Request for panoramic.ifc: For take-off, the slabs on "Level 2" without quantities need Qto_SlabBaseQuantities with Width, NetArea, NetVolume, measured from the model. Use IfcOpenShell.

First a look at what the model holds.

```python
import ifcopenshell
import ifcopenshell.util.element
import ifcopenshell.util.unit

model = ifcopenshell.open("panoramic.ifc")
print(model.schema)
for unit_type in ("LENGTHUNIT", "AREAUNIT", "VOLUMEUNIT"):
    print(unit_type, ifcopenshell.util.unit.calculate_unit_scale(model, unit_type))
storey = next(s for s in model.by_type("IfcBuildingStorey") if s.Name == "Level 2")
slabs = [e for e in ifcopenshell.util.element.get_decomposition(storey) if e.is_a("IfcSlab")]
for e in sorted(slabs, key=lambda e: e.id()):
    print(e.id(), e.is_a(), e.Name, list(ifcopenshell.util.element.get_psets(e, qtos_only=True)), sep=" | ")
```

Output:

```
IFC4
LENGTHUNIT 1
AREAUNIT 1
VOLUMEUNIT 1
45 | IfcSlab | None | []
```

```python
import ifcopenshell
import ifcopenshell.api.pset
import ifcopenshell.geom
import ifcopenshell.util.element
import ifcopenshell.util.shape
import ifcopenshell.util.unit

model = ifcopenshell.open("panoramic.ifc")
unit_scale = ifcopenshell.util.unit.calculate_unit_scale(model)
area_scale = ifcopenshell.util.unit.calculate_unit_scale(model, "AREAUNIT")
volume_scale = ifcopenshell.util.unit.calculate_unit_scale(model, "VOLUMEUNIT")
settings = ifcopenshell.geom.settings()

storey = next(s for s in model.by_type("IfcBuildingStorey") if s.Name == "Level 2")
slabs = [e for e in ifcopenshell.util.element.get_decomposition(storey) if e.is_a("IfcSlab")]

for e in sorted(slabs, key=lambda e: e.id()):
    if ifcopenshell.util.element.get_psets(e, qtos_only=True, should_inherit=False):
        continue
    # Geometry comes back in metres, in the element's own axes.
    shape = ifcopenshell.geom.create_shape(settings, e)
    values = {
        "Width": ifcopenshell.util.shape.get_z(shape.geometry) / unit_scale,
        "NetArea": ifcopenshell.util.shape.get_footprint_area(shape.geometry) / area_scale,
        "NetVolume": ifcopenshell.util.shape.get_volume(shape.geometry) / volume_scale,
    }
    qto = ifcopenshell.api.pset.add_qto(model, product=e, name="Qto_SlabBaseQuantities")
    ifcopenshell.api.pset.edit_qto(model, qto=qto, properties=values)
    print(e.id(), {k: round(v, 3) for k, v in values.items()})

model.write("panoramic_edited.ifc")
```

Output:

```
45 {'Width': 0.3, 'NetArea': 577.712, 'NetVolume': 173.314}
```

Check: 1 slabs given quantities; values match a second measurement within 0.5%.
